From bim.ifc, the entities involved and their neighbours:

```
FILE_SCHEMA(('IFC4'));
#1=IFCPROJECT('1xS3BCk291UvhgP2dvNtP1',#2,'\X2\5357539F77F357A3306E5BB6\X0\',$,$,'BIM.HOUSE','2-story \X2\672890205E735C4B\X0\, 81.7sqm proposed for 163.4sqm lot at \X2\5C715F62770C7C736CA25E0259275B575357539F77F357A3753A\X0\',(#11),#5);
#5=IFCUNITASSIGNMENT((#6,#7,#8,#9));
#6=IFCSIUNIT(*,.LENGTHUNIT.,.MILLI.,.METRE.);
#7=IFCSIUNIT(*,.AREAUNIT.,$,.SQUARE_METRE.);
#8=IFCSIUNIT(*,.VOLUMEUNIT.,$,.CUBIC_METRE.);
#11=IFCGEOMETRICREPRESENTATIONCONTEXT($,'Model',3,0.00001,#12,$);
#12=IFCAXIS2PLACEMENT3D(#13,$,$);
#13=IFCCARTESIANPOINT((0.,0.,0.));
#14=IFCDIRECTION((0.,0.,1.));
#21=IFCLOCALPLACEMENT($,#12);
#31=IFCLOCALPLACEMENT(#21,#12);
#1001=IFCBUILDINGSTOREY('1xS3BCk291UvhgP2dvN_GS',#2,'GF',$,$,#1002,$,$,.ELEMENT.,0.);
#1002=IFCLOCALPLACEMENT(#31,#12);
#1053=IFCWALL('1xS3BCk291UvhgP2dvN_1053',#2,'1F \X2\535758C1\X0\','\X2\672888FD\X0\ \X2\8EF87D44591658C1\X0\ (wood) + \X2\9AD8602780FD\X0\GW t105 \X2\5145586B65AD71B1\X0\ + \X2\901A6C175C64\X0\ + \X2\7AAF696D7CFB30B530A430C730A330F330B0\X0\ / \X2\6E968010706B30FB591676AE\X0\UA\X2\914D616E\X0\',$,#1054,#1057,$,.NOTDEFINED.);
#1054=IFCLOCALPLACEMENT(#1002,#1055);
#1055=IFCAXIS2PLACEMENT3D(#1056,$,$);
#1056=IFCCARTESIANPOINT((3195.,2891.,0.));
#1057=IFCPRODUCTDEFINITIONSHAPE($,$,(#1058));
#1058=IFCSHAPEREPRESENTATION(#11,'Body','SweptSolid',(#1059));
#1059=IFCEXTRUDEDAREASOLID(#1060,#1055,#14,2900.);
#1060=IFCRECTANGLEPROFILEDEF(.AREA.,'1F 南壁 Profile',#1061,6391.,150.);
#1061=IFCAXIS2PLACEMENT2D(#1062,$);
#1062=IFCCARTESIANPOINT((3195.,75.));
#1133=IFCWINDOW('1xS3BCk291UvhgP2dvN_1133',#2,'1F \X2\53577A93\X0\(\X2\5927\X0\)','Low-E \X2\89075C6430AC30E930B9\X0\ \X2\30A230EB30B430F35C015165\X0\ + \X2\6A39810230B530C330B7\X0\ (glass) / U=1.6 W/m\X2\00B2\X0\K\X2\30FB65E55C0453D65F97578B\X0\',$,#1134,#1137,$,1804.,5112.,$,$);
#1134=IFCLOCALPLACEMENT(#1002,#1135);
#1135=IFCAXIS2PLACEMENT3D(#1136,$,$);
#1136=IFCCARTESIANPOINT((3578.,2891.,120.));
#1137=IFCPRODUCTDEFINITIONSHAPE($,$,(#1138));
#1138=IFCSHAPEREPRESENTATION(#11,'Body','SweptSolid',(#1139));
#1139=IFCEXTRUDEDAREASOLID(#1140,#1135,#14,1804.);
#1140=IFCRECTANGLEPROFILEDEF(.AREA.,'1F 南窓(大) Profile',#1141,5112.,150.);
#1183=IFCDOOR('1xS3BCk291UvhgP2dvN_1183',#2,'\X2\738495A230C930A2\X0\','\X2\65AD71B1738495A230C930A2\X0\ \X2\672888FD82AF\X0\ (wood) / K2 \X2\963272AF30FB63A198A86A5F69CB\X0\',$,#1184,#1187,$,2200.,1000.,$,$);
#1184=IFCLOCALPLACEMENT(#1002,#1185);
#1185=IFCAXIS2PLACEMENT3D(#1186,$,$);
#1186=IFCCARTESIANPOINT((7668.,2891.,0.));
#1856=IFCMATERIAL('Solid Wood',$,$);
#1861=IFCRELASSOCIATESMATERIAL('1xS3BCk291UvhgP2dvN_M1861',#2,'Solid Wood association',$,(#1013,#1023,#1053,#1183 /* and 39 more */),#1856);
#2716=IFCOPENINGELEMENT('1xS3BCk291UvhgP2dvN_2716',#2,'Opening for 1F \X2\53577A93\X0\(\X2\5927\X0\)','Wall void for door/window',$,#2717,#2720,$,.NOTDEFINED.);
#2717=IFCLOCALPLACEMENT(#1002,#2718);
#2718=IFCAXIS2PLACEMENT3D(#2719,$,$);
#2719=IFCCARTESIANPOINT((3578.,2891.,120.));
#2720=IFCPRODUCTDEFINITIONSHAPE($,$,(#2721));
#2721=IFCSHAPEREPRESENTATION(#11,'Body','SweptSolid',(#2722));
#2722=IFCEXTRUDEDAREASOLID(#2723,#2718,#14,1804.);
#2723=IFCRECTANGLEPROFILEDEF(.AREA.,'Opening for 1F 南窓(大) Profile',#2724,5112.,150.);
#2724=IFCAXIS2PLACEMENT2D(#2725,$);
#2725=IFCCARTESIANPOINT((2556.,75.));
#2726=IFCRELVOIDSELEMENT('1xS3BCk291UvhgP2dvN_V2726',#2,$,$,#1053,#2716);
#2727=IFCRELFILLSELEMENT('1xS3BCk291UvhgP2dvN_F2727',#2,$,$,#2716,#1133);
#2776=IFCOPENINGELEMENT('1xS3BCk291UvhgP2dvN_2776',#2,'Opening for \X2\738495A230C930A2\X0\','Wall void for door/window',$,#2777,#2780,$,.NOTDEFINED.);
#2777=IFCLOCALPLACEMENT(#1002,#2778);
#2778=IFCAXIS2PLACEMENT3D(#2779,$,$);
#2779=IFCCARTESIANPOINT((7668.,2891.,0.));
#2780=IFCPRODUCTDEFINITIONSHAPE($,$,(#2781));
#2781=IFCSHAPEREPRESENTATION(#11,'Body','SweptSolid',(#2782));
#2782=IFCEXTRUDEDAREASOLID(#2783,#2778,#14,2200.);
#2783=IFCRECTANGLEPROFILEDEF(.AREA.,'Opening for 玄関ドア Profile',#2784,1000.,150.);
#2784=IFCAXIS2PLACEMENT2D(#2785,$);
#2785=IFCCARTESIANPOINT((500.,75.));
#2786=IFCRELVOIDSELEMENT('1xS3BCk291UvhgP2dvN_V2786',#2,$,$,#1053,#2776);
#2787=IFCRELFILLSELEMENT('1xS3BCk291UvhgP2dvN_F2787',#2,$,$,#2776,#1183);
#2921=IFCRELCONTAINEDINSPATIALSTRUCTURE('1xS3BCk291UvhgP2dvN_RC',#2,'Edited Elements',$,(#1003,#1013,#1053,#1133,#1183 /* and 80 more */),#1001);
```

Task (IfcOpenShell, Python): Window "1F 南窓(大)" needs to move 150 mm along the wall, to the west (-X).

```python
import ifcopenshell
import ifcopenshell.api.geometry
import ifcopenshell.util.placement
import ifcopenshell.util.unit

model = ifcopenshell.open("bim.ifc")
unit_scale = ifcopenshell.util.unit.calculate_unit_scale(model)

window = model.by_guid("1xS3BCk291UvhgP2dvN_1133")
opening = window.FillsVoids[0].RelatingOpeningElement
wall = opening.VoidsElements[0].RelatingBuildingElement

wall_matrix = ifcopenshell.util.placement.get_local_placement(wall.ObjectPlacement)
shift = wall_matrix[:3, 0] * -0.15 / unit_scale
before = ifcopenshell.util.placement.get_local_placement(window.ObjectPlacement)[:3, 3].copy()

# The window is not placed relative to its opening, so move both.
for product in (opening, window):
    matrix = ifcopenshell.util.placement.get_local_placement(product.ObjectPlacement)
    matrix[:3, 3] += shift
    ifcopenshell.api.geometry.edit_object_placement(model, product=product, matrix=matrix, is_si=False)

after = ifcopenshell.util.placement.get_local_placement(window.ObjectPlacement)[:3, 3]
print("window moved by", (after - before).round(3) + 0.0)

model.write("bim_v2.ifc")
```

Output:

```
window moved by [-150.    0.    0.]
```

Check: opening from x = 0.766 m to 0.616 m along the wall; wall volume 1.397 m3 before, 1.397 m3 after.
